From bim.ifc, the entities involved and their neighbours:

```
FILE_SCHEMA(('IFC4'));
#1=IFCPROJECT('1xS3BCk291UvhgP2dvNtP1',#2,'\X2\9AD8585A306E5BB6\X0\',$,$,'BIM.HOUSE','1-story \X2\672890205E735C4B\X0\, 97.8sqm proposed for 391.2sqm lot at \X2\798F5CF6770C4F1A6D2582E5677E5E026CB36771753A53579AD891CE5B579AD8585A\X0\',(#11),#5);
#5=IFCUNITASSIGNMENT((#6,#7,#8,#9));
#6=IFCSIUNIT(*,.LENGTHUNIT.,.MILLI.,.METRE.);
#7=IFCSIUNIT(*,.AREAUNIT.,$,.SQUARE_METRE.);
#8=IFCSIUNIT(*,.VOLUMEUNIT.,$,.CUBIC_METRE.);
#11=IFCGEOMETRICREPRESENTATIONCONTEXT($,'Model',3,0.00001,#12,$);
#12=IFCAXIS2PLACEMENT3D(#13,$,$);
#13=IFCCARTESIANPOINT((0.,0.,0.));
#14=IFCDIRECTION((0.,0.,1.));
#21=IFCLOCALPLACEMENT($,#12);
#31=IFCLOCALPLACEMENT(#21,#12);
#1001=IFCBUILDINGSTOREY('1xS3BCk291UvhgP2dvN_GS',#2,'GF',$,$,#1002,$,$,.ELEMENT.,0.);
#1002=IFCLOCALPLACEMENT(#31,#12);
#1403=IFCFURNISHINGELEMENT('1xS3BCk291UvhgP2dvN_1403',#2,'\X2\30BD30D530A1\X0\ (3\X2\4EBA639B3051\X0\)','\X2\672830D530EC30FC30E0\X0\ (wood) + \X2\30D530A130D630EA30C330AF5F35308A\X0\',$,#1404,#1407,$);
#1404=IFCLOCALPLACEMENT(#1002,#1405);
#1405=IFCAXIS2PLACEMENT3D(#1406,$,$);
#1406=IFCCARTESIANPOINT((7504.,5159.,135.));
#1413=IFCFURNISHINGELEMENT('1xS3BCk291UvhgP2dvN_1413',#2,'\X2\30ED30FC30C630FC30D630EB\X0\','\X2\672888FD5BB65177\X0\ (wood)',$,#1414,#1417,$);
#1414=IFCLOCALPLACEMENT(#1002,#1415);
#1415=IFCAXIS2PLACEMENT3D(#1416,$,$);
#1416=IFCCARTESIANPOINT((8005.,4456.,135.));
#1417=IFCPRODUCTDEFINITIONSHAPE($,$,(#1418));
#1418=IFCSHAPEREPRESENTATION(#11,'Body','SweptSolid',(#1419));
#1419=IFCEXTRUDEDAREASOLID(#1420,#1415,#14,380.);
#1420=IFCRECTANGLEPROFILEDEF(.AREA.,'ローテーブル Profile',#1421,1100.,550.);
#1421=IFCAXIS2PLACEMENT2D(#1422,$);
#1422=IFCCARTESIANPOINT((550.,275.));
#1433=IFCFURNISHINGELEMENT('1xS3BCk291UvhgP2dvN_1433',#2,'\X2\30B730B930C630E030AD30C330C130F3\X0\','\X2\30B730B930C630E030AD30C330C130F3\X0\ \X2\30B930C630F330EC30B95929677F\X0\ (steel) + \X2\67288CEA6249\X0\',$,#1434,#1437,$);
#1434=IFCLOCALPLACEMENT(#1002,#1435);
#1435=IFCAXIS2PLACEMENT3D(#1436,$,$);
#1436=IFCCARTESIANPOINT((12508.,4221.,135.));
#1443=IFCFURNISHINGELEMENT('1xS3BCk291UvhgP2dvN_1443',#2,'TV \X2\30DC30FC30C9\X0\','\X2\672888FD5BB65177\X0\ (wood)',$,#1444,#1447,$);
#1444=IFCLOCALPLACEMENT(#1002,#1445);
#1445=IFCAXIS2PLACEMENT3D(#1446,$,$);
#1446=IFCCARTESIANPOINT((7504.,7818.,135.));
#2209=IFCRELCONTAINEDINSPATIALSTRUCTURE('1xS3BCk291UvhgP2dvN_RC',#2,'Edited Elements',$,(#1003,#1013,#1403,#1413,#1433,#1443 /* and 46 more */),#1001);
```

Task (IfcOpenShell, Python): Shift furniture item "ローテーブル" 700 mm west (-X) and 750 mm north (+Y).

```python
import ifcopenshell
import ifcopenshell.api.geometry
import ifcopenshell.util.placement

model = ifcopenshell.open("bim.ifc")

item = model.by_guid("1xS3BCk291UvhgP2dvN_1413")
matrix = ifcopenshell.util.placement.get_local_placement(item.ObjectPlacement)
matrix[0, 3] -= 700.0
matrix[1, 3] += 750.0
ifcopenshell.api.geometry.edit_object_placement(model, product=item, matrix=matrix, is_si=False)

print(ifcopenshell.util.placement.get_local_placement(item.ObjectPlacement).round(3) + 0.0)

model.write("bim_updated.ifc")
```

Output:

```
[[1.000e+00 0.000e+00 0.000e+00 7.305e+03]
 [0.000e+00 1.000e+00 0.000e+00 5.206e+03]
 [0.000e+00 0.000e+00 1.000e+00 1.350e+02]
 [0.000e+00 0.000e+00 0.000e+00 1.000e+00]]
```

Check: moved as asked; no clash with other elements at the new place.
